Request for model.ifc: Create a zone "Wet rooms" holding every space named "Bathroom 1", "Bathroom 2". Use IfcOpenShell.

First a look at what the model holds.

```python
import ifcopenshell

model = ifcopenshell.open("model.ifc")
print(model.schema)
seen = {}
for space in model.by_type("IfcSpace"):
    seen[space.LongName] = seen.get(space.LongName, 0) + 1
for name, count in sorted(seen.items(), key=str):
    print(count, "x", name)
print("zones:", [z.Name for z in model.by_type("IfcZone")][:20])
```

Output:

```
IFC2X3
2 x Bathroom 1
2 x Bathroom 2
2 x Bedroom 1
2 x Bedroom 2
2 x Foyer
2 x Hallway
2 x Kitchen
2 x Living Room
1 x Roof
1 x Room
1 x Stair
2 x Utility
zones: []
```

```python
import ifcopenshell
import ifcopenshell.api.group
import ifcopenshell.api.root

model = ifcopenshell.open("model.ifc")

names = {"Bathroom 1", "Bathroom 2"}
spaces = [s for s in model.by_type("IfcSpace") if s.LongName in names]

zone = ifcopenshell.api.root.create_entity(model, ifc_class="IfcZone", name="Wet rooms")
ifcopenshell.api.group.assign_group(model, products=spaces, group=zone)
print(len(spaces), "spaces in", zone.Name)

model.write("model_rev.ifc")
```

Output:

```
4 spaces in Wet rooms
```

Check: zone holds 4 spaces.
